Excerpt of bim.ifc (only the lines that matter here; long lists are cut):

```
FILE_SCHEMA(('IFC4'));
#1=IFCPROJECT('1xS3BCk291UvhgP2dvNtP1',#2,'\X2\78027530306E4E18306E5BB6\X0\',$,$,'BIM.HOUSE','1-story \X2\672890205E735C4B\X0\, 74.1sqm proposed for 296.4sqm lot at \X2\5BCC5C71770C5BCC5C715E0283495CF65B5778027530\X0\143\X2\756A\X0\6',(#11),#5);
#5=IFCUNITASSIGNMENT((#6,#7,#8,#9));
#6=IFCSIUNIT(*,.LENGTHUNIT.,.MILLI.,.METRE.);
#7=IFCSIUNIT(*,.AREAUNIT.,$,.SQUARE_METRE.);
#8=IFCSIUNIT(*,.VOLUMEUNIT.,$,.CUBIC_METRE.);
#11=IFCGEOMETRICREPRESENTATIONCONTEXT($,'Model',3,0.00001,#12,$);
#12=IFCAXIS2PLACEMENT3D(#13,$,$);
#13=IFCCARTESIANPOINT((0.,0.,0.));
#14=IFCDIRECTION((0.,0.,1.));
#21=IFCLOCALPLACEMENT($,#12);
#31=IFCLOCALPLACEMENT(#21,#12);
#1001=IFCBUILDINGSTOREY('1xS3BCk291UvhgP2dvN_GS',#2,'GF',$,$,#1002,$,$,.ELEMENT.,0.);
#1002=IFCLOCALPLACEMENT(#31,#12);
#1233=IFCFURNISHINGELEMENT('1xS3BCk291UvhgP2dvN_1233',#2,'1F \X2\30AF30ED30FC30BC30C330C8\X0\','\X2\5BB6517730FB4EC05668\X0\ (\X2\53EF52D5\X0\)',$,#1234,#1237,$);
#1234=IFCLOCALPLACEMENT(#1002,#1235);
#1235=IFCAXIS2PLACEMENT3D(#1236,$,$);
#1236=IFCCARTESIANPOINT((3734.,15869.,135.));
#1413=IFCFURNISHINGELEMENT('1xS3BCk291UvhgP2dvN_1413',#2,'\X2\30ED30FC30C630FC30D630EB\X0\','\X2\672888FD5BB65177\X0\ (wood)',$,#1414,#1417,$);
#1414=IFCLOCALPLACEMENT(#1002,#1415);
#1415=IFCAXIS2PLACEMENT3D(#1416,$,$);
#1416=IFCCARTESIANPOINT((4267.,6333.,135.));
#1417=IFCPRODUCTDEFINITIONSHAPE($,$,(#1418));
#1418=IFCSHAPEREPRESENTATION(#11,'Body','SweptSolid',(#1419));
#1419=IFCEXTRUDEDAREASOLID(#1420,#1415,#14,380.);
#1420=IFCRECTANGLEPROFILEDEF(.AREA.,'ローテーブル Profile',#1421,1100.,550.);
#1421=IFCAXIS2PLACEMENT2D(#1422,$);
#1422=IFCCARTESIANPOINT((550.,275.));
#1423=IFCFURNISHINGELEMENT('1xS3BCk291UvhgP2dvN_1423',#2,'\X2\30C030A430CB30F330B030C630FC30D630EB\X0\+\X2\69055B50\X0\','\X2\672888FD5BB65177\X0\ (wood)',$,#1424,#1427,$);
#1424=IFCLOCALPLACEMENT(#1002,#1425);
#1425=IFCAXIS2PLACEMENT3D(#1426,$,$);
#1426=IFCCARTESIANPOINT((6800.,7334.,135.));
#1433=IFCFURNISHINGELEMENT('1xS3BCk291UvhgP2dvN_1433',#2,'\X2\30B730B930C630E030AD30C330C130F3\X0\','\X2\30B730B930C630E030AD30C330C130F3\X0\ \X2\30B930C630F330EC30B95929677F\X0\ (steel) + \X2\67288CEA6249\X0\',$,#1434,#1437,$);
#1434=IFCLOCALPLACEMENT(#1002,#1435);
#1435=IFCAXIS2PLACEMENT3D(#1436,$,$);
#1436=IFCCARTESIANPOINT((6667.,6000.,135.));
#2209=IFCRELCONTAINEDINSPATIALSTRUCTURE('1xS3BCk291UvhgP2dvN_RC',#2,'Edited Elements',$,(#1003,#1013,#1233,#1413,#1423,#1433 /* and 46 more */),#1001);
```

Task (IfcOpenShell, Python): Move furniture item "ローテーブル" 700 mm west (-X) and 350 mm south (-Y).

```python
import ifcopenshell
import ifcopenshell.api.geometry
import ifcopenshell.util.placement

model = ifcopenshell.open("bim.ifc")

item = model.by_guid("1xS3BCk291UvhgP2dvN_1413")
matrix = ifcopenshell.util.placement.get_local_placement(item.ObjectPlacement)
matrix[0, 3] -= 700.0
matrix[1, 3] -= 350.0
ifcopenshell.api.geometry.edit_object_placement(model, product=item, matrix=matrix, is_si=False)

print(ifcopenshell.util.placement.get_local_placement(item.ObjectPlacement).round(3) + 0.0)

model.write("bim_updated.ifc")
```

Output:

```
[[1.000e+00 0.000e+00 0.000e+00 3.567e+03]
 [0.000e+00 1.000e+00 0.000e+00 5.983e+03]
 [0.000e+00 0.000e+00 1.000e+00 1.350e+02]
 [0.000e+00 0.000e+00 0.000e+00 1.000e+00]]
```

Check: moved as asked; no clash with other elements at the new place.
